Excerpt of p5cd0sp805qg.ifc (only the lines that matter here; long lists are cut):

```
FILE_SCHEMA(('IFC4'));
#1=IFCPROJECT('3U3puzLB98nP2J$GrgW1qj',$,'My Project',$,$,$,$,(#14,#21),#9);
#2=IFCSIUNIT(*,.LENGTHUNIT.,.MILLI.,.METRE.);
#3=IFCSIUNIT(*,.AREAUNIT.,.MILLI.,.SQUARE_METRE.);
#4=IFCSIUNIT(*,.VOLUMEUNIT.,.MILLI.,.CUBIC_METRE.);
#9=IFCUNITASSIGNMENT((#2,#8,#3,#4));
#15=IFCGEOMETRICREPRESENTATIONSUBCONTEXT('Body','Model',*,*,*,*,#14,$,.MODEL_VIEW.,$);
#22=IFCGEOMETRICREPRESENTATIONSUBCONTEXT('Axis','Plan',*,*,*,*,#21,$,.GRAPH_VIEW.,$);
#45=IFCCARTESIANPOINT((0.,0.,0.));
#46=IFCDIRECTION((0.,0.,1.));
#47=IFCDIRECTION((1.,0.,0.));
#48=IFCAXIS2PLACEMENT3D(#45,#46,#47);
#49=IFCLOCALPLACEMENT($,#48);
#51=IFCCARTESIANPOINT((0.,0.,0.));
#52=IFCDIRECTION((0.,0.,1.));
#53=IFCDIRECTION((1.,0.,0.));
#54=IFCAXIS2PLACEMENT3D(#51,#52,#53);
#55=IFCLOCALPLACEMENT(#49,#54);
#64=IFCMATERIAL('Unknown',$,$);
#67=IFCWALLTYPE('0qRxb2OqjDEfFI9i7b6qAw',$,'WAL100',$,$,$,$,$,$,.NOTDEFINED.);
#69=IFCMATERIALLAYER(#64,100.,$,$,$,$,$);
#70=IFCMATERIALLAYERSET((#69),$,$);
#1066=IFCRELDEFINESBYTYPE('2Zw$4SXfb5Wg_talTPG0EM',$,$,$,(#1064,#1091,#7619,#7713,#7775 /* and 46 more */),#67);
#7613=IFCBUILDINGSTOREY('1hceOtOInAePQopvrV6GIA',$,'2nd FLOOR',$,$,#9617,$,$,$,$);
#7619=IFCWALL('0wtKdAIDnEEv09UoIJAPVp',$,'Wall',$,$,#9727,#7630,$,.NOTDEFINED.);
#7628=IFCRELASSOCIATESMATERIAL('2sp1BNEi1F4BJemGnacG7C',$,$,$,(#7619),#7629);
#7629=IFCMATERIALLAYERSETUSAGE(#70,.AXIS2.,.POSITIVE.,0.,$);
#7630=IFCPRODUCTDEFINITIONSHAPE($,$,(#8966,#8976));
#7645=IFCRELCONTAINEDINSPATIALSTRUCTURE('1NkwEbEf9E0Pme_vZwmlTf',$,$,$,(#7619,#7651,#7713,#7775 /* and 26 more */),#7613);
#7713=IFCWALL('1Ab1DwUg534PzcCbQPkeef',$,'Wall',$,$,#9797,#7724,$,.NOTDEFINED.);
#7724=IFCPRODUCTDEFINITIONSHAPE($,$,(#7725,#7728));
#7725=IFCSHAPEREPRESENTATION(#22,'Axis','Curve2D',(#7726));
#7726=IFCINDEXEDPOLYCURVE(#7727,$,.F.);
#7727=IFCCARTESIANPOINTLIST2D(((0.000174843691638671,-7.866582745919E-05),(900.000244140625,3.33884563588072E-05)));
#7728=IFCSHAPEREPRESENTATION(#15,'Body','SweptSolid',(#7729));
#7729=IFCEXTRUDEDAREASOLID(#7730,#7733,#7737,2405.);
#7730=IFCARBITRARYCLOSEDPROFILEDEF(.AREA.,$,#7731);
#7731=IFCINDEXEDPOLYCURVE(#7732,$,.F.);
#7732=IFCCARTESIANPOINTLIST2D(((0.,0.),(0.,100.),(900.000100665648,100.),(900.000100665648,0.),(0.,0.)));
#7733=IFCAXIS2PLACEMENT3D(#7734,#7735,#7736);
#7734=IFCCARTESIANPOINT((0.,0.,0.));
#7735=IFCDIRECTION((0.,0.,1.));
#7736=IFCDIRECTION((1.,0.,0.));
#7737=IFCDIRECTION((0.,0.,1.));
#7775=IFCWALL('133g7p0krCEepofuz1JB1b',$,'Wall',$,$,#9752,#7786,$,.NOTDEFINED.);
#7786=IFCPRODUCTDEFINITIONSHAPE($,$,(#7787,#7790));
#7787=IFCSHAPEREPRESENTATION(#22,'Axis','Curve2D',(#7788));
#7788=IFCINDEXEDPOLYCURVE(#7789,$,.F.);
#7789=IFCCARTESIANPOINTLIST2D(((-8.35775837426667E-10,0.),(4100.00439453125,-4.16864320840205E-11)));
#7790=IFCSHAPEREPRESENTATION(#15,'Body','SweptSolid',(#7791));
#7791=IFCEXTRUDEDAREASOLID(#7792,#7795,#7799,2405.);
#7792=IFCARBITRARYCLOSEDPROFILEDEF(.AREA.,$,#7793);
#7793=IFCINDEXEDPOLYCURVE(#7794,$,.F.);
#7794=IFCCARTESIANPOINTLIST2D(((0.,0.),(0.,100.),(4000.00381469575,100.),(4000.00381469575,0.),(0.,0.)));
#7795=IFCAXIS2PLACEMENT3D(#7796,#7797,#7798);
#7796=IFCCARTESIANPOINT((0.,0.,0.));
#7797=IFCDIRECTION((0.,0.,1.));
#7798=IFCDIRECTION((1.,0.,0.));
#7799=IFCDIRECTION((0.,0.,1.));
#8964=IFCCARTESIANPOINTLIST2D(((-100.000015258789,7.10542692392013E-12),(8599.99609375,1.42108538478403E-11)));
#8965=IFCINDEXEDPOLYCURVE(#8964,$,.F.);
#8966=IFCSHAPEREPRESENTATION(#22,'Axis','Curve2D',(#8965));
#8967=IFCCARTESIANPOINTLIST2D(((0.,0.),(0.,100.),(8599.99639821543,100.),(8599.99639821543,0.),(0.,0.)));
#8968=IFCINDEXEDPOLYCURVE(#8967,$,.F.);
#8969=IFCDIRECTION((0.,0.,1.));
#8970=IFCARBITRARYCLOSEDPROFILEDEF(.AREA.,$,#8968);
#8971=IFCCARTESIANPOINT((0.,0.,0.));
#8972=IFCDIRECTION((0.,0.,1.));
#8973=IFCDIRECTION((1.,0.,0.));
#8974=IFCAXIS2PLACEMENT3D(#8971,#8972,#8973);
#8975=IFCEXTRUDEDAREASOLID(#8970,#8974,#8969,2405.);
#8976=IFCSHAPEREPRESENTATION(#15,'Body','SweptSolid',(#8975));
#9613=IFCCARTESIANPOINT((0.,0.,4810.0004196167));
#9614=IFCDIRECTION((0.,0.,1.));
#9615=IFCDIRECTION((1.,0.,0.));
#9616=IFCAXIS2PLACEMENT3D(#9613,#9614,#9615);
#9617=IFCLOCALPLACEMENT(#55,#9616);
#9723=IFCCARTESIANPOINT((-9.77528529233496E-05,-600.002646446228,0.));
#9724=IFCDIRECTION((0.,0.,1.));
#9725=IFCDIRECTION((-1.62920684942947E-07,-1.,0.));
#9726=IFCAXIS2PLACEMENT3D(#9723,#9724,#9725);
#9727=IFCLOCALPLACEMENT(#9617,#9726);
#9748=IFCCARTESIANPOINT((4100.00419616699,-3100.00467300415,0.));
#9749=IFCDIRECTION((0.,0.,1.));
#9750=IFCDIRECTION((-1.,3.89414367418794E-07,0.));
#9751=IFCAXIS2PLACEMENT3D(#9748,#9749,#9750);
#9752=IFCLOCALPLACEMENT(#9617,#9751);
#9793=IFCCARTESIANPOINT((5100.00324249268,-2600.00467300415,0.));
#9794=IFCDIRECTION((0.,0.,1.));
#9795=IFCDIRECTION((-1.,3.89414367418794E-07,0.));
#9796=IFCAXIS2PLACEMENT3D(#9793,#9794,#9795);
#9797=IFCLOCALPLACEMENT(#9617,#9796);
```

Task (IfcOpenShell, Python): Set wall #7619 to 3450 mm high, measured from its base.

```python
import ifcopenshell
import ifcopenshell.geom
import ifcopenshell.util.representation
import ifcopenshell.util.shape

model = ifcopenshell.open("p5cd0sp805qg.ifc")
settings = ifcopenshell.geom.settings()


def volume(element):
    """Net volume in cubic metres, openings subtracted."""
    shape = ifcopenshell.geom.create_shape(settings, element)
    return ifcopenshell.util.shape.get_volume(shape.geometry)


wall = model.by_guid("0wtKdAIDnEEv09UoIJAPVp")
before = volume(wall)

body = ifcopenshell.util.representation.get_representation(wall, "Model", "Body")
solid = body.Items[0]
old_height = solid.Depth
solid.Depth = 3450.0
after = volume(wall)

print(f"height {old_height:g} -> {solid.Depth:g}, volume {before:.3f} -> {after:.3f} m3")

model.write("p5cd0sp805qg-out.ifc")
```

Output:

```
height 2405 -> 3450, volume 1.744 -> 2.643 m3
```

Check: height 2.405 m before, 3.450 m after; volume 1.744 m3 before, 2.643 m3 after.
